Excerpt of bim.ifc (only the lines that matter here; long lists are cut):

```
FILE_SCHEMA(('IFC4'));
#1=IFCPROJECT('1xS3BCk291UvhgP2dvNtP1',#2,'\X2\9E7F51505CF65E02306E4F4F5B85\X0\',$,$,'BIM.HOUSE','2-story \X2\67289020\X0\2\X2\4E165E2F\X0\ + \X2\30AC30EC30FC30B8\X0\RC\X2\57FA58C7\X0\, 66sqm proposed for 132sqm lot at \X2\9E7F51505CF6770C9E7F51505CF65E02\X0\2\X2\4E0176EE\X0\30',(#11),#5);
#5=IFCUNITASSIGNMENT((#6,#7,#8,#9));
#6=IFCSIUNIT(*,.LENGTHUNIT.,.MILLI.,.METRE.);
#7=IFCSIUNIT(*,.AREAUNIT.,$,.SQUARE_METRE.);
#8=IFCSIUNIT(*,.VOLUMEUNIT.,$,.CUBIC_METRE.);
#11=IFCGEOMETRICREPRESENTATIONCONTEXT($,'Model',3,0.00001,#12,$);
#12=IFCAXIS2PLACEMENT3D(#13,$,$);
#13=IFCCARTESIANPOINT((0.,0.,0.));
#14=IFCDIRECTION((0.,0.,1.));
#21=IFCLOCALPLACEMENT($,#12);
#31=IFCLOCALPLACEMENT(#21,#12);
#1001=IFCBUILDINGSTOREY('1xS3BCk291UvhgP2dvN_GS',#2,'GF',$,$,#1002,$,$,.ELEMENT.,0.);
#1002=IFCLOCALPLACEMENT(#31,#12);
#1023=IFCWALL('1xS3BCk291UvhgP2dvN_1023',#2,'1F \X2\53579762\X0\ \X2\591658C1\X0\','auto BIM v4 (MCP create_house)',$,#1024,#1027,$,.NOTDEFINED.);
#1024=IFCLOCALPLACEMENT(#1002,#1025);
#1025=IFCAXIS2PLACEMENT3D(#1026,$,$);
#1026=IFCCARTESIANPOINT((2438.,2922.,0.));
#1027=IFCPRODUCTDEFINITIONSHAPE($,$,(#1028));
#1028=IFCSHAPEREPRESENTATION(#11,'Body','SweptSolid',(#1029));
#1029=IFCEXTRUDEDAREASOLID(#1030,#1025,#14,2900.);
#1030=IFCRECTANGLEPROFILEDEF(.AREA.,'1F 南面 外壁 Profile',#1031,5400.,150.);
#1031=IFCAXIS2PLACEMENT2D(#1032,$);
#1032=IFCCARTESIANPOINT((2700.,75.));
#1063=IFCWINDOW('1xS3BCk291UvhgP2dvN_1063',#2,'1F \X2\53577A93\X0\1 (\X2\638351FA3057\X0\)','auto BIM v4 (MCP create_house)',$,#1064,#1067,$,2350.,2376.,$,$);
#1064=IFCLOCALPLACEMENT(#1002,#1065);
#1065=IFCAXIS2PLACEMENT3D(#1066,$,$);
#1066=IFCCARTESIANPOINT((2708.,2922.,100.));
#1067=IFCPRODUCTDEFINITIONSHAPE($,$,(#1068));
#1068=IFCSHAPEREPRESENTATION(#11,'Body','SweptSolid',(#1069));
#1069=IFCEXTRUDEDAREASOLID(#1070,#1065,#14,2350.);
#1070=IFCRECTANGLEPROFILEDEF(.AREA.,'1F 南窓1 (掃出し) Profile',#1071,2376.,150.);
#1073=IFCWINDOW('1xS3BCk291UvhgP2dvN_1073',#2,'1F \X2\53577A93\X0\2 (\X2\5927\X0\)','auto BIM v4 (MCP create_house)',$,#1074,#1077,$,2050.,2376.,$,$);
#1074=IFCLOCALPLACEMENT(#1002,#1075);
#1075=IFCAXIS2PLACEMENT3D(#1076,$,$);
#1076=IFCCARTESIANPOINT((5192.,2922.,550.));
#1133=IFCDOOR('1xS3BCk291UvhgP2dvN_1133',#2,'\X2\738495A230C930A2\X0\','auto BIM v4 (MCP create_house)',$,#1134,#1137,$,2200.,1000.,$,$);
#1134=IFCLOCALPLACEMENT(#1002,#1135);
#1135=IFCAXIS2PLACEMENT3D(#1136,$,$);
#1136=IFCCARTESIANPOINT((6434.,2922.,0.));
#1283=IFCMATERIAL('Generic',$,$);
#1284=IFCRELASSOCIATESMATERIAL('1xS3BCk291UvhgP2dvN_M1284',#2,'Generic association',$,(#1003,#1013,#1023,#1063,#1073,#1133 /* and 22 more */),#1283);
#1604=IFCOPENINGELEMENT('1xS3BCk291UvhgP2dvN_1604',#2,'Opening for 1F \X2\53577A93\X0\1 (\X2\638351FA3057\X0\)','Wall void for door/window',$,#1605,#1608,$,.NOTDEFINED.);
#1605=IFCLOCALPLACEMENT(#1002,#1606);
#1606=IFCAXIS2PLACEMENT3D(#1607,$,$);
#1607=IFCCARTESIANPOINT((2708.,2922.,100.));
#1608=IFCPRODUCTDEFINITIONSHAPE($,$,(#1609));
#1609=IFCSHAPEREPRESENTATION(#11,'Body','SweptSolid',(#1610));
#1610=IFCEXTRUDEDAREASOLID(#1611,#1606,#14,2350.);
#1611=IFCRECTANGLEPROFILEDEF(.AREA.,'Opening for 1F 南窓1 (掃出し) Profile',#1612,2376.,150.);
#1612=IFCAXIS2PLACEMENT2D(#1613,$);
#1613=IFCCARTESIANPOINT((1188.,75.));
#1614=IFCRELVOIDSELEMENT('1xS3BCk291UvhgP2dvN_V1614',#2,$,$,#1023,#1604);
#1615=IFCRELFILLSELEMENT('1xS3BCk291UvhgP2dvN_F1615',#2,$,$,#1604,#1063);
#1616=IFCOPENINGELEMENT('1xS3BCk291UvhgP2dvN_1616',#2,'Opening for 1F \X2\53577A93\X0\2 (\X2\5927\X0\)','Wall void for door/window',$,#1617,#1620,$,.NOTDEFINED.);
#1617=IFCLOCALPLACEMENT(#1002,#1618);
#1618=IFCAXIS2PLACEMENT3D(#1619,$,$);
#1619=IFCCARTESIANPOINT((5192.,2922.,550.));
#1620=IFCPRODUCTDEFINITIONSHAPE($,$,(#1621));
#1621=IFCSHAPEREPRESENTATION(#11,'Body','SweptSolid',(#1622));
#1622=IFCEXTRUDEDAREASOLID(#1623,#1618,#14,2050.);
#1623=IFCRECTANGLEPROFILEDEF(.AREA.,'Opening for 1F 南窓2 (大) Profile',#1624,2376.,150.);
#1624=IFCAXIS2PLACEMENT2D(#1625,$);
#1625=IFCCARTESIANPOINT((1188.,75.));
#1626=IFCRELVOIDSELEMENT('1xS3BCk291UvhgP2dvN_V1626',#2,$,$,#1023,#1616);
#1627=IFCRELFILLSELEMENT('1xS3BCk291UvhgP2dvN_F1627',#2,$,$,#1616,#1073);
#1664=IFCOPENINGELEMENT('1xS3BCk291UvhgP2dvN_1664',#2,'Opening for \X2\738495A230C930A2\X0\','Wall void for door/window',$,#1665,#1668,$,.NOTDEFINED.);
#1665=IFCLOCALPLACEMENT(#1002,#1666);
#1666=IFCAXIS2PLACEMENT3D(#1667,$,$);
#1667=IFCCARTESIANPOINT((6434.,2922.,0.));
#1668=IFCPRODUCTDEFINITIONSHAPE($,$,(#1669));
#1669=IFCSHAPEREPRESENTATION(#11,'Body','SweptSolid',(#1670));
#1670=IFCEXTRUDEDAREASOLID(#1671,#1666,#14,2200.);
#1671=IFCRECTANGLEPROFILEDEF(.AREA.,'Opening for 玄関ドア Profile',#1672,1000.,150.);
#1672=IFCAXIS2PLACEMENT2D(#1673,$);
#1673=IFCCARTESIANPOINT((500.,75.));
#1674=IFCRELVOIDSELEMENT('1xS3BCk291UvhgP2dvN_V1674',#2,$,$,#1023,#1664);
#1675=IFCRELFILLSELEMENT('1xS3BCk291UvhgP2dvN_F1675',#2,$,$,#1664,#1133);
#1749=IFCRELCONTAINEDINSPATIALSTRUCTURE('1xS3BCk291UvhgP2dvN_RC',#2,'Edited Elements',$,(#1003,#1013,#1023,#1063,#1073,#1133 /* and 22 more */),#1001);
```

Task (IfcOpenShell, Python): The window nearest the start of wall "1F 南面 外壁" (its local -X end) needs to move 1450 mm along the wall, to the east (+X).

```python
import ifcopenshell
import ifcopenshell.api.geometry
import ifcopenshell.util.placement
import ifcopenshell.util.unit

model = ifcopenshell.open("bim.ifc")
unit_scale = ifcopenshell.util.unit.calculate_unit_scale(model)

window = model.by_id(1063)
opening = window.FillsVoids[0].RelatingOpeningElement
wall = opening.VoidsElements[0].RelatingBuildingElement

wall_matrix = ifcopenshell.util.placement.get_local_placement(wall.ObjectPlacement)
shift = wall_matrix[:3, 0] * 1.45 / unit_scale
before = ifcopenshell.util.placement.get_local_placement(window.ObjectPlacement)[:3, 3].copy()

# The window is not placed relative to its opening, so move both.
for product in (opening, window):
    matrix = ifcopenshell.util.placement.get_local_placement(product.ObjectPlacement)
    matrix[:3, 3] += shift
    ifcopenshell.api.geometry.edit_object_placement(model, product=product, matrix=matrix, is_si=False)

after = ifcopenshell.util.placement.get_local_placement(window.ObjectPlacement)[:3, 3]
print("window moved by", (after - before).round(3) + 0.0)

model.write("bim_updated.ifc")
```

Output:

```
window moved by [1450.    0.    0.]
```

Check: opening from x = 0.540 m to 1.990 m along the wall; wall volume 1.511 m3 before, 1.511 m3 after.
